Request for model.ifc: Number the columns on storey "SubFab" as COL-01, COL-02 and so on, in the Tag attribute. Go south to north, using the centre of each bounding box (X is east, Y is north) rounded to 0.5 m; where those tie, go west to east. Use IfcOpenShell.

First a look at what the model holds.

```python
import ifcopenshell
import ifcopenshell.util.element
import ifcopenshell.util.placement

model = ifcopenshell.open("model.ifc")
print(model.schema)
storey = next(s for s in model.by_type("IfcBuildingStorey") if s.Name == "SubFab")
columns = [e for e in ifcopenshell.util.element.get_decomposition(storey) if e.is_a("IfcColumn")]
for e in sorted(columns, key=lambda e: e.id()):
    origin = ifcopenshell.util.placement.get_local_placement(e.ObjectPlacement)[:3, 3]
    print(e.id(), e.Tag, e.Name, origin.round(2) + 0.0, sep=" | ")
```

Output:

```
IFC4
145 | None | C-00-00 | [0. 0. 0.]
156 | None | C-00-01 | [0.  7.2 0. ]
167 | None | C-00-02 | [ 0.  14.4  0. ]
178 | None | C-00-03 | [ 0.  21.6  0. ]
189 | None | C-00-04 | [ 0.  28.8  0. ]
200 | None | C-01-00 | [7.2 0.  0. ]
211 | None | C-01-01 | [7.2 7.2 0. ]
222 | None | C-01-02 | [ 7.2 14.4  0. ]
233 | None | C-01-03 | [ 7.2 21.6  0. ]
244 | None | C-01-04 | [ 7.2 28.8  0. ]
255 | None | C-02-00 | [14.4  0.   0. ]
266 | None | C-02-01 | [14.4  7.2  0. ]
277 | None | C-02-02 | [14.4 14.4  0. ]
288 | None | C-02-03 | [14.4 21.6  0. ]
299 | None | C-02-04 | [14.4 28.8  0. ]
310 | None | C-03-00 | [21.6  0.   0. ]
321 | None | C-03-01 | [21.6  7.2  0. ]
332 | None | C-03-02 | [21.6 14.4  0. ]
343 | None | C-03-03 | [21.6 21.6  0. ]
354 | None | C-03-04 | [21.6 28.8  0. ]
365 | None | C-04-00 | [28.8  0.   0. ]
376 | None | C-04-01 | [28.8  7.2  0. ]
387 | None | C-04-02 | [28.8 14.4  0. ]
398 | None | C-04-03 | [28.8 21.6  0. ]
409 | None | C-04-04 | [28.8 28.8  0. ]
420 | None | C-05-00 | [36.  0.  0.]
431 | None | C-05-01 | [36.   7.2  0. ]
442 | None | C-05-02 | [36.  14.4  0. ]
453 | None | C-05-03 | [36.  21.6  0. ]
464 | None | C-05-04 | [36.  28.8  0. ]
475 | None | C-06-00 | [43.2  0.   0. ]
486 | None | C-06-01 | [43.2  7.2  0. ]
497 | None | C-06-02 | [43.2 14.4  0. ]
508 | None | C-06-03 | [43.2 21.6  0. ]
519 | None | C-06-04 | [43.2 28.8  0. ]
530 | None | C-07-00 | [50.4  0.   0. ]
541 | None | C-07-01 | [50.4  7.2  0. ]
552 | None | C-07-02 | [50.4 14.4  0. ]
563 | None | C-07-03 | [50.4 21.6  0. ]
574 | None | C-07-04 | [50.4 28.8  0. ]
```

```python
import ifcopenshell
import ifcopenshell.geom
import ifcopenshell.util.element
import ifcopenshell.util.shape

model = ifcopenshell.open("model.ifc")
settings = ifcopenshell.geom.settings()
settings.set("use-world-coords", True)


def centre(element):
    shape = ifcopenshell.geom.create_shape(settings, element)
    return ifcopenshell.util.shape.get_bbox_centroid(shape.geometry)


storey = next(s for s in model.by_type("IfcBuildingStorey") if s.Name == "SubFab")
columns = [e for e in ifcopenshell.util.element.get_decomposition(storey) if e.is_a("IfcColumn")]

# Insertion points can sit at a corner or the storey origin, so sort by the geometry (in metres).
centres = {e: centre(e) for e in columns}
columns.sort(key=lambda e: (round(centres[e][1] / 0.5), centres[e][0]))

for i, e in enumerate(columns, start=1):
    number = f"COL-{i:02d}"
    e.Tag = number
    print(e.id(), number)

model.write("model-out.ifc")
```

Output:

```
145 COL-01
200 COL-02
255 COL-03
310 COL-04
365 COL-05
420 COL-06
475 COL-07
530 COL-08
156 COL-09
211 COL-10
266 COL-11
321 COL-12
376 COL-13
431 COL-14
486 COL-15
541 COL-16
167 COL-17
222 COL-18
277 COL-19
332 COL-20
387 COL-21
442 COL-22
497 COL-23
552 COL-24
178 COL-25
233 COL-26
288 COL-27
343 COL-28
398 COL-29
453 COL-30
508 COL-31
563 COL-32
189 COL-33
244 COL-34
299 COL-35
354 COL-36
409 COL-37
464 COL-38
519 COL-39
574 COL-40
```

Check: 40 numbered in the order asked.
